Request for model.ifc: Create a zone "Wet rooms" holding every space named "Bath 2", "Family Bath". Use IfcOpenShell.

First a look at what the model holds.

```python
import ifcopenshell

model = ifcopenshell.open("model.ifc")
print(model.schema)
seen = {}
for space in model.by_type("IfcSpace"):
    seen[space.LongName] = seen.get(space.LongName, 0) + 1
for name, count in sorted(seen.items(), key=str):
    print(count, "x", name)
print("zones:", [z.Name for z in model.by_type("IfcZone")][:20])
```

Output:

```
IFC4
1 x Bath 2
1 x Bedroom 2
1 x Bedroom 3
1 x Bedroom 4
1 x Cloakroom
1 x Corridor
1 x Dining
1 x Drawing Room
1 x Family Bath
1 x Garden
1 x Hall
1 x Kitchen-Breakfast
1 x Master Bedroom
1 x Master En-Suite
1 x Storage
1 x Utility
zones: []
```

```python
import ifcopenshell
import ifcopenshell.api.group
import ifcopenshell.api.root

model = ifcopenshell.open("model.ifc")

names = {"Bath 2", "Family Bath"}
spaces = [s for s in model.by_type("IfcSpace") if s.LongName in names]

zone = ifcopenshell.api.root.create_entity(model, ifc_class="IfcZone", name="Wet rooms")
ifcopenshell.api.group.assign_group(model, products=spaces, group=zone)
print(len(spaces), "spaces in", zone.Name)

model.write("model_edited.ifc")
```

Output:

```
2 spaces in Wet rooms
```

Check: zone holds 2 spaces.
